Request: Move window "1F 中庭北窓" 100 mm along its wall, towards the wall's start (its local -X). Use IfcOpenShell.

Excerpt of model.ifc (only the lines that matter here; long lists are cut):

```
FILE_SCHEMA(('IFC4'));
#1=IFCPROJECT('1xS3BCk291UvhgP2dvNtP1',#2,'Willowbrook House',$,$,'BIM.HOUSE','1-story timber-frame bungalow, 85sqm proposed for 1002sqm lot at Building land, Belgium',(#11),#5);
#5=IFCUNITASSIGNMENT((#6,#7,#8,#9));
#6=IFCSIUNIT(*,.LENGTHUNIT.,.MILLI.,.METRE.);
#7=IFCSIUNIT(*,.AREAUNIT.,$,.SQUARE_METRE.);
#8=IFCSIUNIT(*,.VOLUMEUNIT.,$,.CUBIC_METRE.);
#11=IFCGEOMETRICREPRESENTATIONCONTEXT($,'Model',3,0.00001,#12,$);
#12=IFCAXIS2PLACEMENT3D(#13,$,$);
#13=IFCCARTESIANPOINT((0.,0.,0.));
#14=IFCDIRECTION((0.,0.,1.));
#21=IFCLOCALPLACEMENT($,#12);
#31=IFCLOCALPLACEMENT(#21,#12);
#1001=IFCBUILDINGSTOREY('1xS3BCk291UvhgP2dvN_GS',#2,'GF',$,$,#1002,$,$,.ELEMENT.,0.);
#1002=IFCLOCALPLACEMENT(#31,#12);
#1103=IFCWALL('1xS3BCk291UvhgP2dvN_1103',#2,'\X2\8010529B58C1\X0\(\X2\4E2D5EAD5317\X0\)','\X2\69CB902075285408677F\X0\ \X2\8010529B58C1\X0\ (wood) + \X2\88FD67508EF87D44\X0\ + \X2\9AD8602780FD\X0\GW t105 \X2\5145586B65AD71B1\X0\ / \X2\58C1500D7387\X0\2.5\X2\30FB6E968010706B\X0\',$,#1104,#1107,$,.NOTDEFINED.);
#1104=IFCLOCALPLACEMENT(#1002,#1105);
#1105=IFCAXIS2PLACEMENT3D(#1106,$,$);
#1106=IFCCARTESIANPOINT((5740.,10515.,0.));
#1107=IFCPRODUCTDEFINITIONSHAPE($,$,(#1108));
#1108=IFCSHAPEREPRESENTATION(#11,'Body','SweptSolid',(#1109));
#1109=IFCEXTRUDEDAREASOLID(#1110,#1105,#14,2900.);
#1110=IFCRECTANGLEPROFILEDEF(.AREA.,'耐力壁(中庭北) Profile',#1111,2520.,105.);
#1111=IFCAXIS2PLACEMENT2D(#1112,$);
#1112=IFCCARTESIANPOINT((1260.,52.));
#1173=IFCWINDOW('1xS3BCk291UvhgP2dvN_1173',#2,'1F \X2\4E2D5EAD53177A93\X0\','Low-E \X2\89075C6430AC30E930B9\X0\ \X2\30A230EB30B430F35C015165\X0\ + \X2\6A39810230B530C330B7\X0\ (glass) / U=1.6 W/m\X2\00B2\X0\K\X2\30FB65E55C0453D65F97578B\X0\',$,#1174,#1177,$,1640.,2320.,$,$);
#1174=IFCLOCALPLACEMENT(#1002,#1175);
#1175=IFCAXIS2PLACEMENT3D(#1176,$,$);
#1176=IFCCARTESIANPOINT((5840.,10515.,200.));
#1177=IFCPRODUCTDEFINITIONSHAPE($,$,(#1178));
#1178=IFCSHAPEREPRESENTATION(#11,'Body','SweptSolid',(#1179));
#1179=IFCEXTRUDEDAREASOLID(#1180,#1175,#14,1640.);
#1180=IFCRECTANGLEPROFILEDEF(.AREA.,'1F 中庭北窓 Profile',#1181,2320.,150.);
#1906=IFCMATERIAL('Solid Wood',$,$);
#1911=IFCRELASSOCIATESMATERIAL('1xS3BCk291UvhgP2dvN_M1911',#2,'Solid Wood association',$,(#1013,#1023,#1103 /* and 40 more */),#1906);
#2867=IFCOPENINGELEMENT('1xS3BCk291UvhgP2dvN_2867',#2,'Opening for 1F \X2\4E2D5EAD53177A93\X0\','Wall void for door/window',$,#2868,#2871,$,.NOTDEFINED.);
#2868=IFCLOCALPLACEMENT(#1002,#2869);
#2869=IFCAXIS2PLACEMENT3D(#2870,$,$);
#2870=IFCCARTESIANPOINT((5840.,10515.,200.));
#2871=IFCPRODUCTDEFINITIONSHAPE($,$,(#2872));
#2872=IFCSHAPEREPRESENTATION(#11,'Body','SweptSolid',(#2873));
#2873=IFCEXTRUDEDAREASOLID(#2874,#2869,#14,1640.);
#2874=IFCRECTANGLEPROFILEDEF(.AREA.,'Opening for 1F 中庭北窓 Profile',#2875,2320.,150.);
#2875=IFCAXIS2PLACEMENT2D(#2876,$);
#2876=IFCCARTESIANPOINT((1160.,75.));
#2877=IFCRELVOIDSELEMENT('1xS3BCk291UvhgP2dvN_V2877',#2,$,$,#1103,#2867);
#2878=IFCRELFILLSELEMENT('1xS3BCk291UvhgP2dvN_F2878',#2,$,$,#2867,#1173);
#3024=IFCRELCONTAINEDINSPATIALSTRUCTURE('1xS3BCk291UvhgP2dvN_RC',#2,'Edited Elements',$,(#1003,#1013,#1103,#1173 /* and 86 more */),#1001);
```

```python
import ifcopenshell
import ifcopenshell.api.geometry
import ifcopenshell.util.placement

model = ifcopenshell.open("model.ifc")

window = model.by_guid("1xS3BCk291UvhgP2dvN_1173")
opening = window.FillsVoids[0].RelatingOpeningElement
wall = opening.VoidsElements[0].RelatingBuildingElement

wall_matrix = ifcopenshell.util.placement.get_local_placement(wall.ObjectPlacement)
shift = wall_matrix[:3, 0] * -100.0
before = ifcopenshell.util.placement.get_local_placement(window.ObjectPlacement)[:3, 3].copy()

# The window is not placed relative to its opening, so move both.
for product in (opening, window):
    matrix = ifcopenshell.util.placement.get_local_placement(product.ObjectPlacement)
    matrix[:3, 3] += shift
    ifcopenshell.api.geometry.edit_object_placement(model, product=product, matrix=matrix, is_si=False)

after = ifcopenshell.util.placement.get_local_placement(window.ObjectPlacement)[:3, 3]
print("window moved by", (after - before).round(3) + 0.0)

model.write("model_v2.ifc")
```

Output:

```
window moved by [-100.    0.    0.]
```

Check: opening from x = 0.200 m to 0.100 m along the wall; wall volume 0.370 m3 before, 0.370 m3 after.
